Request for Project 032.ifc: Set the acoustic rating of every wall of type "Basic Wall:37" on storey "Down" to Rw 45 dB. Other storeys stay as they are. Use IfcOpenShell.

First a look at what the model holds.

```python
import ifcopenshell
import ifcopenshell.util.element

model = ifcopenshell.open("Project 032.ifc")
print(model.schema)
storey = next(s for s in model.by_type("IfcBuildingStorey") if s.Name == "Down")
walls = [e for e in ifcopenshell.util.element.get_decomposition(storey) if e.is_a("IfcWall")]
seen = {}
for e in walls:
    element_type = ifcopenshell.util.element.get_type(e)
    key = (element_type.Name if element_type != e and element_type else None, ifcopenshell.util.element.get_pset(e, "Pset_WallCommon", "AcousticRating"))
    seen[key] = seen.get(key, 0) + 1
for (name, value), count in sorted(seen.items(), key=str):
    print(count, "x", name, "|", value)
```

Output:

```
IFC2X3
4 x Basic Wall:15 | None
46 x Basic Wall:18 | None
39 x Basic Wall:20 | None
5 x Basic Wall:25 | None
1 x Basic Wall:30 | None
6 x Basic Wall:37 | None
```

```python
import ifcopenshell
import ifcopenshell.api.pset
import ifcopenshell.util.element

model = ifcopenshell.open("Project 032.ifc")

storey = next(s for s in model.by_type("IfcBuildingStorey") if s.Name == "Down")
walls = [e for e in ifcopenshell.util.element.get_decomposition(storey) if e.is_a("IfcWall")]

count = 0
for e in walls:
    element_type = ifcopenshell.util.element.get_type(e)
    if element_type in (None, e) or element_type.Name != "Basic Wall:37":
        continue
    # add_pset returns the element's existing set when there is one.
    pset = ifcopenshell.api.pset.add_pset(model, product=e, name="Pset_WallCommon")
    ifcopenshell.api.pset.edit_pset(model, pset=pset, properties={"AcousticRating": "Rw 45 dB"})
    count += 1

print(count, "walls updated")

model.write("Project 032-out.ifc")
```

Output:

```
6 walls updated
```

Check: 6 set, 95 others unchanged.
